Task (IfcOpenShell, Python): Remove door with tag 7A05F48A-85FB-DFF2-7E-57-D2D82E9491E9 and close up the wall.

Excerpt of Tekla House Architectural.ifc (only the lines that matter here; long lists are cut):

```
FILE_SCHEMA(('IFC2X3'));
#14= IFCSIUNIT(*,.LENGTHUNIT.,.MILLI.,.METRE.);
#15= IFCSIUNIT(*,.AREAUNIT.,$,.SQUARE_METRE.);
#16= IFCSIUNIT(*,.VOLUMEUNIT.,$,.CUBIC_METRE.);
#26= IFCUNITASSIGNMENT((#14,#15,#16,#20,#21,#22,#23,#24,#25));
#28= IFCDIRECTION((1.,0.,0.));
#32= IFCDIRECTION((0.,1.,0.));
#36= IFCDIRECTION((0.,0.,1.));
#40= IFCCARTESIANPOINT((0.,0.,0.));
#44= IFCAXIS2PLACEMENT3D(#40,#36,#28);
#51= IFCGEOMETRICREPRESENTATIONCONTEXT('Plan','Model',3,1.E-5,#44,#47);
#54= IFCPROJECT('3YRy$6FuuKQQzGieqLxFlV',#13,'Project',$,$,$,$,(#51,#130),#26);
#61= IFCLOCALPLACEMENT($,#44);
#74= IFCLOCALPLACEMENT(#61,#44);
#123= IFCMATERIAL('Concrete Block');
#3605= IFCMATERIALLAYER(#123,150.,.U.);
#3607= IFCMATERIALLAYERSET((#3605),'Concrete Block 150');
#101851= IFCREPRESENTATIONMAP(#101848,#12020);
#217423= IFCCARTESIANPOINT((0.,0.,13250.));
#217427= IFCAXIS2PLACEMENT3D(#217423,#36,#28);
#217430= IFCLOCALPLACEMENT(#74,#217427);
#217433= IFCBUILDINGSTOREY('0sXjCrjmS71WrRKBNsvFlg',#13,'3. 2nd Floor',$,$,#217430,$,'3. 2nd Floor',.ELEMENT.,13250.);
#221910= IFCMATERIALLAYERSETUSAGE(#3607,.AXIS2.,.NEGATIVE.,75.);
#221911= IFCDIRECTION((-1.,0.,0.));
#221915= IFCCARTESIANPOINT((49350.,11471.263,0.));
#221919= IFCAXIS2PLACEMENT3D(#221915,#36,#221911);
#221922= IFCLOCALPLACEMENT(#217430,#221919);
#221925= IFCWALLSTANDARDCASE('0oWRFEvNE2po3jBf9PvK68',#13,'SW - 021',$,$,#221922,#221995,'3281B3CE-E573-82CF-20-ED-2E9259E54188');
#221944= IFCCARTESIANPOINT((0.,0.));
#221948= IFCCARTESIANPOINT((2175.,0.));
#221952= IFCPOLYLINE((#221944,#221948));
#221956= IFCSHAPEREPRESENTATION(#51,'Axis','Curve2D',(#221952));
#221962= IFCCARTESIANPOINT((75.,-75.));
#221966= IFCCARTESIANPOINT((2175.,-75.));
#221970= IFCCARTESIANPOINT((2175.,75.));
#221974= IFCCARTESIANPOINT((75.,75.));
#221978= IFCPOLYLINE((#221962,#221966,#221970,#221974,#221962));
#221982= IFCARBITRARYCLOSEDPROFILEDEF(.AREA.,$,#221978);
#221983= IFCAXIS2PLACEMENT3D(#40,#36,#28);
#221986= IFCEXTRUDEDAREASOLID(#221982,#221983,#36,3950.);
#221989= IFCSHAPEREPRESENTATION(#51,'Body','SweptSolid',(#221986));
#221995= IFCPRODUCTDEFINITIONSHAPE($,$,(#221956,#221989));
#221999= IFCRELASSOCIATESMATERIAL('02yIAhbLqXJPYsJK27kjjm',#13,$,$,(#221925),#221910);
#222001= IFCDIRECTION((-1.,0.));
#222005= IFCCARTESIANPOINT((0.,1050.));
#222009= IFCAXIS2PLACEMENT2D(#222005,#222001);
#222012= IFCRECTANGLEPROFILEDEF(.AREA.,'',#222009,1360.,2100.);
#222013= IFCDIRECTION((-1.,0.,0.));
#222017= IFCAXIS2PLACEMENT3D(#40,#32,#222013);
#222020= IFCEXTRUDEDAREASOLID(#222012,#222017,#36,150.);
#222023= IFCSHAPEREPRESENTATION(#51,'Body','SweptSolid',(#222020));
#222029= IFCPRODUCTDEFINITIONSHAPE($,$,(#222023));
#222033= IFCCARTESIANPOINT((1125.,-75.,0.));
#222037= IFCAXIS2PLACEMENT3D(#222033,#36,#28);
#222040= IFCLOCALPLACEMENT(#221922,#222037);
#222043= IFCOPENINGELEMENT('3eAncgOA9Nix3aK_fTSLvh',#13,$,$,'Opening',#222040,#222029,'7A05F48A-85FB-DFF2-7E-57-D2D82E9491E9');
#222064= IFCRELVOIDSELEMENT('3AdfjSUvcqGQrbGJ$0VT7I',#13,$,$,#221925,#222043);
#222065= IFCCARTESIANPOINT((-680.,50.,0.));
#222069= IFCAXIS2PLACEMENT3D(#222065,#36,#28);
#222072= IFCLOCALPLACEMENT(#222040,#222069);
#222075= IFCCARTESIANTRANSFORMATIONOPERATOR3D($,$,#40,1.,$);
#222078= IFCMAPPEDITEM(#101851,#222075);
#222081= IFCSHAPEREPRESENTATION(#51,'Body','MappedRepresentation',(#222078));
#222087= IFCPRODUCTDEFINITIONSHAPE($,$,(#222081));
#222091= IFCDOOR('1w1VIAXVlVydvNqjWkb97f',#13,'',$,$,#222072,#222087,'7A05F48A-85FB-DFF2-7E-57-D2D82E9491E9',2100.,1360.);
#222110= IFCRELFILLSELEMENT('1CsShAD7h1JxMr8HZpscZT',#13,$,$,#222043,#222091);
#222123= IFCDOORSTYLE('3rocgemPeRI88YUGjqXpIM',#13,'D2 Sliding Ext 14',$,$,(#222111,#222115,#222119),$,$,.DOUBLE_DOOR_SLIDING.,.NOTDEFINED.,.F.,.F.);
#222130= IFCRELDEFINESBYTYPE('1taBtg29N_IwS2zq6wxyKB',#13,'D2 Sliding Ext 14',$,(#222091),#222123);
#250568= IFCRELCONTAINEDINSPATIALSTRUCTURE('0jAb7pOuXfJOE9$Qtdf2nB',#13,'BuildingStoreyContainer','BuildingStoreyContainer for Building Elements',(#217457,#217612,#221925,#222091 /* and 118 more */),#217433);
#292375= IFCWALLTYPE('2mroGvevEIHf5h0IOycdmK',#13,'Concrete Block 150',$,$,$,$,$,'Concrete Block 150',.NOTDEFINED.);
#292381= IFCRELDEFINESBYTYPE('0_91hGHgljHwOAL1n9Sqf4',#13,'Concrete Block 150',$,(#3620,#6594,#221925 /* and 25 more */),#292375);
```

```python
import ifcopenshell
import ifcopenshell.api.feature
import ifcopenshell.api.root
import ifcopenshell.geom
import ifcopenshell.util.shape

model = ifcopenshell.open("Tekla House Architectural.ifc")
settings = ifcopenshell.geom.settings()


def volume(element):
    """Net volume in cubic metres, openings subtracted."""
    shape = ifcopenshell.geom.create_shape(settings, element)
    return ifcopenshell.util.shape.get_volume(shape.geometry)


door = model.by_guid("1w1VIAXVlVydvNqjWkb97f")
opening = door.FillsVoids[0].RelatingOpeningElement
wall = opening.VoidsElements[0].RelatingBuildingElement
before = volume(wall)

ifcopenshell.api.root.remove_product(model, product=door)
ifcopenshell.api.feature.remove_feature(model, feature=opening)

after = volume(wall)

print(f"wall volume {before:.3f} -> {after:.3f} m3")

model.write("Tekla House Architectural-out.ifc")
```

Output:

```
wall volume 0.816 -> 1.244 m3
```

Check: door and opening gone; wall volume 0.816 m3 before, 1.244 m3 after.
